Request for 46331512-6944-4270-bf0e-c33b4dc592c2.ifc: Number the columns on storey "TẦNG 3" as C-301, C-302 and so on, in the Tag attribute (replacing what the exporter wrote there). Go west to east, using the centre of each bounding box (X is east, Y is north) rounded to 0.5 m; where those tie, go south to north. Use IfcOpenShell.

First a look at what the model holds.

```python
import ifcopenshell
import ifcopenshell.util.element
import ifcopenshell.util.placement

model = ifcopenshell.open("46331512-6944-4270-bf0e-c33b4dc592c2.ifc")
print(model.schema)
storey = next(s for s in model.by_type("IfcBuildingStorey") if s.Name == "TẦNG 3")
columns = [e for e in ifcopenshell.util.element.get_decomposition(storey) if e.is_a("IfcColumn")]
for e in sorted(columns, key=lambda e: e.id()):
    origin = ifcopenshell.util.placement.get_local_placement(e.ObjectPlacement)[:3, 3]
    print(e.id(), e.Tag, e.Name, origin.round(2) + 0.0, sep=" | ")
```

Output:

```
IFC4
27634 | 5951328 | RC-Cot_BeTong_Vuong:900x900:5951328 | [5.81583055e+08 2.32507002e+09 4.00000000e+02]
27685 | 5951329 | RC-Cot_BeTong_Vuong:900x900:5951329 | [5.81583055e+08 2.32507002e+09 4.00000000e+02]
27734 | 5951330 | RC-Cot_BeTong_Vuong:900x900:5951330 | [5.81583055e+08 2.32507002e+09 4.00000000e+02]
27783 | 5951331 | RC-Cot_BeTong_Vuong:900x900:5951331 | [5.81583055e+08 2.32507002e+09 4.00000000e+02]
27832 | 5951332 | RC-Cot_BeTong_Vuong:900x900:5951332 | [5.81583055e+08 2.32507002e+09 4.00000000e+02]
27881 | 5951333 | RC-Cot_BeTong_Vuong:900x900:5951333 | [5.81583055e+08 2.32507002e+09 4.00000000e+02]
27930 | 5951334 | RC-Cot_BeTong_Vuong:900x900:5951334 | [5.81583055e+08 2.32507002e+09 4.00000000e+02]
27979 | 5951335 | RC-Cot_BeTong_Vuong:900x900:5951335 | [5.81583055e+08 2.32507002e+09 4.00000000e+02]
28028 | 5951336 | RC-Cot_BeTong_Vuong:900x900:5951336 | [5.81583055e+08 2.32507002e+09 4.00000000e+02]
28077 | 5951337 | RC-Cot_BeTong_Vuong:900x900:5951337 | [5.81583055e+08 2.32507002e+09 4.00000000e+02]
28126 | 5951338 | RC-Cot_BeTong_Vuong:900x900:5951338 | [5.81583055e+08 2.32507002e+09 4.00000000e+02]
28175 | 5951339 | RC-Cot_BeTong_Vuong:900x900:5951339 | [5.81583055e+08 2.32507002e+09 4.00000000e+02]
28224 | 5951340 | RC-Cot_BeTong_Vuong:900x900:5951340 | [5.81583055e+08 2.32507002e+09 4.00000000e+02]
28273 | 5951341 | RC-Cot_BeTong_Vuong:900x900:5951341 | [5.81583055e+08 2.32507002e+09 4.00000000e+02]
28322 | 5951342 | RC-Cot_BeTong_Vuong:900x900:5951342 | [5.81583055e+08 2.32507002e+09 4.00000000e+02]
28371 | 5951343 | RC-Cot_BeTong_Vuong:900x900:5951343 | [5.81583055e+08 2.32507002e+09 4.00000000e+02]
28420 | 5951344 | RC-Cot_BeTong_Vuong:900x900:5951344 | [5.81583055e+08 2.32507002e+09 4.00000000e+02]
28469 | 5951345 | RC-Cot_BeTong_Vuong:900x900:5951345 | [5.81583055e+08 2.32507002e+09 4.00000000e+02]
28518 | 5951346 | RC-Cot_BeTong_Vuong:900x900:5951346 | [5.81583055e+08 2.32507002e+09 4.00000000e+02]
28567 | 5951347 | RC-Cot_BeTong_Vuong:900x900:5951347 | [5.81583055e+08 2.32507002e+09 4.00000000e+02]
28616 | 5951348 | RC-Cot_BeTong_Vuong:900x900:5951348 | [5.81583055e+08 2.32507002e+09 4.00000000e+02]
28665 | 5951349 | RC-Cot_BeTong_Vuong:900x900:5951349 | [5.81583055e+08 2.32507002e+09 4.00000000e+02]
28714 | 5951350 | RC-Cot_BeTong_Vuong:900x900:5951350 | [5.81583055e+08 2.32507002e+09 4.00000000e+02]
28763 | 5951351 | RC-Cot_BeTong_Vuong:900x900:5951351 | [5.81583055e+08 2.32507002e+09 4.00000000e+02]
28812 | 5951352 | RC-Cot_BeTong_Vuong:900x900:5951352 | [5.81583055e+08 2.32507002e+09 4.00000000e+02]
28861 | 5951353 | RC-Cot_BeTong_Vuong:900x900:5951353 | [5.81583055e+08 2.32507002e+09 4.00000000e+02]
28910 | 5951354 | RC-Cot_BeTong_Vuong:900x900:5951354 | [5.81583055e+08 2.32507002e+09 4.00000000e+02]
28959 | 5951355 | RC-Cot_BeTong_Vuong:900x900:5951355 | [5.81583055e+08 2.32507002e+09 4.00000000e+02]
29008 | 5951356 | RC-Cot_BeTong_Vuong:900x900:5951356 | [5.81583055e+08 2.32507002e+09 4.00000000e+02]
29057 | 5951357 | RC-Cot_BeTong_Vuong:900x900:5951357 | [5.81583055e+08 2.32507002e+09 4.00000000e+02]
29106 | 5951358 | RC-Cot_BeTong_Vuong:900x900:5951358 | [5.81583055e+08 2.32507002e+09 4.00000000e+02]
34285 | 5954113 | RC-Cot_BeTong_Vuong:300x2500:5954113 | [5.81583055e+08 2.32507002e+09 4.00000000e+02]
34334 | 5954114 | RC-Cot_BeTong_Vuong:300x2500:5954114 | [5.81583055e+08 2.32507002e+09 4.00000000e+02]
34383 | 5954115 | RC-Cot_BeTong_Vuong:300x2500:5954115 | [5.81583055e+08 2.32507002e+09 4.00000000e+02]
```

```python
import ifcopenshell
import ifcopenshell.geom
import ifcopenshell.util.element
import ifcopenshell.util.shape

model = ifcopenshell.open("46331512-6944-4270-bf0e-c33b4dc592c2.ifc")
settings = ifcopenshell.geom.settings()
settings.set("use-world-coords", True)


def centre(element):
    shape = ifcopenshell.geom.create_shape(settings, element)
    return ifcopenshell.util.shape.get_bbox_centroid(shape.geometry)


storey = next(s for s in model.by_type("IfcBuildingStorey") if s.Name == "TẦNG 3")
columns = [e for e in ifcopenshell.util.element.get_decomposition(storey) if e.is_a("IfcColumn")]

# Insertion points can sit at a corner or the storey origin, so sort by the geometry (in metres).
centres = {e: centre(e) for e in columns}
columns.sort(key=lambda e: (round(centres[e][0] / 0.5), centres[e][1]))

for i, e in enumerate(columns, start=1):
    number = f"C-3{i:02d}"
    e.Tag = number
    print(e.id(), number)

model.write("46331512-6944-4270-bf0e-c33b4dc592c2_edited.ifc")
```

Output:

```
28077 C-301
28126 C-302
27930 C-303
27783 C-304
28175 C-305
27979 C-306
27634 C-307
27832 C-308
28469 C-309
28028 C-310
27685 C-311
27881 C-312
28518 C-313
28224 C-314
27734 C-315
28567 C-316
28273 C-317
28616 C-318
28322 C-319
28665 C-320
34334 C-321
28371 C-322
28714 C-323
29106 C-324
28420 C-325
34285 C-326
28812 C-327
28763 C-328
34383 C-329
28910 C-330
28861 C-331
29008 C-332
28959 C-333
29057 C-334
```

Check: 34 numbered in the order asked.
